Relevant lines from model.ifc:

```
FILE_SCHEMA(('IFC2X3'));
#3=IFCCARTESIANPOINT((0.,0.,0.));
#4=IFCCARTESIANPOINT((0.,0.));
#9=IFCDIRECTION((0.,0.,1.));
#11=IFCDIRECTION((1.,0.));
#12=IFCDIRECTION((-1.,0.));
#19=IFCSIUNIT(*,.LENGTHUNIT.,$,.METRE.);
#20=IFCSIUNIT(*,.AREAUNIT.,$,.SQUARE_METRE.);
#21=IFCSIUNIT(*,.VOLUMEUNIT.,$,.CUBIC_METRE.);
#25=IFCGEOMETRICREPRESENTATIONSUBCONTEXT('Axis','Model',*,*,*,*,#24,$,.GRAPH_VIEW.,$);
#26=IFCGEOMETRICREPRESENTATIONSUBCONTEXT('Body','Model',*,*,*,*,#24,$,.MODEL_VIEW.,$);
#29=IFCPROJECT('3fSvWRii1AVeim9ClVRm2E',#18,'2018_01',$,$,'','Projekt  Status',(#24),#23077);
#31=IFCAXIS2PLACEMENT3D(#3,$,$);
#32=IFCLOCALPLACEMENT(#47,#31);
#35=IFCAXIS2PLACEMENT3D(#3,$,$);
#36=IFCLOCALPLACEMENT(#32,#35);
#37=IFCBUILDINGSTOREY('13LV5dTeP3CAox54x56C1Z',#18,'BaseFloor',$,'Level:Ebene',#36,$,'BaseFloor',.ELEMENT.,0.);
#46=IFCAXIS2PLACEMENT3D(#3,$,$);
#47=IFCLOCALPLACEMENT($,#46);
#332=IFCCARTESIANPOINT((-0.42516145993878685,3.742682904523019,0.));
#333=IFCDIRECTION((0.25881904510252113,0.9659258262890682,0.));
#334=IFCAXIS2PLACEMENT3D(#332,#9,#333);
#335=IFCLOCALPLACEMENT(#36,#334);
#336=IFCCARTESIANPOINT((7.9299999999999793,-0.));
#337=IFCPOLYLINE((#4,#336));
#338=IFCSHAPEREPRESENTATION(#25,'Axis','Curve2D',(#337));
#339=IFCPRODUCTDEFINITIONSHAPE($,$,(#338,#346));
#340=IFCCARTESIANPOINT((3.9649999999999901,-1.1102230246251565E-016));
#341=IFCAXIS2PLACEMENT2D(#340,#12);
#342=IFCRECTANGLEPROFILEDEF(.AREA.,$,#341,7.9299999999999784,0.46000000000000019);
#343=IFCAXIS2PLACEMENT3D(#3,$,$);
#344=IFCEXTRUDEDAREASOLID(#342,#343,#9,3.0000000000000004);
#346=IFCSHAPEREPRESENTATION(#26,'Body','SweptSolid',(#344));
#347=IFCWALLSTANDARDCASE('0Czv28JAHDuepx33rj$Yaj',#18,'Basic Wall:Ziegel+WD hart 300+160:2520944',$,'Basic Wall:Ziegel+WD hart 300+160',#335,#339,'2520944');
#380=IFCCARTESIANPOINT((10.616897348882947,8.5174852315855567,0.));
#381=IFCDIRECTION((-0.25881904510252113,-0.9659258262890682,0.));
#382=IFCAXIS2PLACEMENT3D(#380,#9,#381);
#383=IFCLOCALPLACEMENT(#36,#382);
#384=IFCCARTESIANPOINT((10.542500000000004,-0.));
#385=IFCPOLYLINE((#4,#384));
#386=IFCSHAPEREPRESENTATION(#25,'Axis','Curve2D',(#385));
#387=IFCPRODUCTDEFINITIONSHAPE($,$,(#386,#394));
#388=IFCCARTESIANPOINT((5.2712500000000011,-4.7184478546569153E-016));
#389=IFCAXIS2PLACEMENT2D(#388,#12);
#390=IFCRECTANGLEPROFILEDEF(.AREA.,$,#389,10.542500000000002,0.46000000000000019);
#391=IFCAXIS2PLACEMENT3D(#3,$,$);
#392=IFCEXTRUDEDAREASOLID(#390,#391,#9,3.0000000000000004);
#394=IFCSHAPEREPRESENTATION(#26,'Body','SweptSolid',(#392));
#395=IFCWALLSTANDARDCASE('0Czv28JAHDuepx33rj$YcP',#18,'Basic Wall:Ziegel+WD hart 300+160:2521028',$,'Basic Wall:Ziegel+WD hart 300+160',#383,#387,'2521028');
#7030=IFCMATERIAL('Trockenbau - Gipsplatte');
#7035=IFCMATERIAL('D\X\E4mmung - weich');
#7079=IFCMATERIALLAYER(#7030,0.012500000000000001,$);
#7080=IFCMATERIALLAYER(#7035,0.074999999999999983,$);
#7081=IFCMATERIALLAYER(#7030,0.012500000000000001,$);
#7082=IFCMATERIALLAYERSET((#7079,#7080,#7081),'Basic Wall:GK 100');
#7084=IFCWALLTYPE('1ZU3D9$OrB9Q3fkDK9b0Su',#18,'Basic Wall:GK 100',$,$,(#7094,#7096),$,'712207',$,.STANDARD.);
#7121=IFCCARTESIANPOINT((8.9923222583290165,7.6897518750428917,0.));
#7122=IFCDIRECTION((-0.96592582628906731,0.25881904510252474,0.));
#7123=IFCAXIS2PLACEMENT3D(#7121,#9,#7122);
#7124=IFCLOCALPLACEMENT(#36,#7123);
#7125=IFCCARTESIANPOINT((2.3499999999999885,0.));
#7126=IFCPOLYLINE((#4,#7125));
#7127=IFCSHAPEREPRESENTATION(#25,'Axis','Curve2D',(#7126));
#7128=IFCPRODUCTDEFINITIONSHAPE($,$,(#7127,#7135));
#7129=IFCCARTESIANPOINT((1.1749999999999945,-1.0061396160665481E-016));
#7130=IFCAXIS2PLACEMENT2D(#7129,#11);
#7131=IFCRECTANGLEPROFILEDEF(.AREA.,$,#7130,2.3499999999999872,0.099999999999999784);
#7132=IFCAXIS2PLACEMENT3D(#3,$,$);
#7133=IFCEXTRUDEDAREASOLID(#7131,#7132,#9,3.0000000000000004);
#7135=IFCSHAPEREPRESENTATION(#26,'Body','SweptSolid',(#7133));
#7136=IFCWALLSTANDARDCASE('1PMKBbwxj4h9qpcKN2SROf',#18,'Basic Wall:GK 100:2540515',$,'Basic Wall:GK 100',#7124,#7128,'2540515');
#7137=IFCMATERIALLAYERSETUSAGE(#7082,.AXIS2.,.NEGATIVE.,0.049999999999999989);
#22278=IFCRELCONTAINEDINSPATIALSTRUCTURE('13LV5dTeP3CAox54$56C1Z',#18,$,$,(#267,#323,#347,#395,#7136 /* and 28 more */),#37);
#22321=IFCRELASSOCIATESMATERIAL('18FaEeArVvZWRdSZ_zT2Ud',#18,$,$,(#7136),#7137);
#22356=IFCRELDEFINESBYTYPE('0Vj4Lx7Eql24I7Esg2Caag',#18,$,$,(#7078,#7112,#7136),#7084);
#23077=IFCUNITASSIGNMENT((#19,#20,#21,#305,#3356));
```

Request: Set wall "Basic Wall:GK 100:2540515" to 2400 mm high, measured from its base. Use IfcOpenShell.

```python
import ifcopenshell
import ifcopenshell.geom
import ifcopenshell.util.representation
import ifcopenshell.util.shape

model = ifcopenshell.open("model.ifc")
settings = ifcopenshell.geom.settings()


def volume(element):
    """Net volume in cubic metres, openings subtracted."""
    shape = ifcopenshell.geom.create_shape(settings, element)
    return ifcopenshell.util.shape.get_volume(shape.geometry)


wall = model.by_guid("1PMKBbwxj4h9qpcKN2SROf")
before = volume(wall)

body = ifcopenshell.util.representation.get_representation(wall, "Model", "Body")
solid = body.Items[0]
old_height = solid.Depth
solid.Depth = 2.4
after = volume(wall)

print(f"height {old_height:g} -> {solid.Depth:g}, volume {before:.3f} -> {after:.3f} m3")

model.write("model-out.ifc")
```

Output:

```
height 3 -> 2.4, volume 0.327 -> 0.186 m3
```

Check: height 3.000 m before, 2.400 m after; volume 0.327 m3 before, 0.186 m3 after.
